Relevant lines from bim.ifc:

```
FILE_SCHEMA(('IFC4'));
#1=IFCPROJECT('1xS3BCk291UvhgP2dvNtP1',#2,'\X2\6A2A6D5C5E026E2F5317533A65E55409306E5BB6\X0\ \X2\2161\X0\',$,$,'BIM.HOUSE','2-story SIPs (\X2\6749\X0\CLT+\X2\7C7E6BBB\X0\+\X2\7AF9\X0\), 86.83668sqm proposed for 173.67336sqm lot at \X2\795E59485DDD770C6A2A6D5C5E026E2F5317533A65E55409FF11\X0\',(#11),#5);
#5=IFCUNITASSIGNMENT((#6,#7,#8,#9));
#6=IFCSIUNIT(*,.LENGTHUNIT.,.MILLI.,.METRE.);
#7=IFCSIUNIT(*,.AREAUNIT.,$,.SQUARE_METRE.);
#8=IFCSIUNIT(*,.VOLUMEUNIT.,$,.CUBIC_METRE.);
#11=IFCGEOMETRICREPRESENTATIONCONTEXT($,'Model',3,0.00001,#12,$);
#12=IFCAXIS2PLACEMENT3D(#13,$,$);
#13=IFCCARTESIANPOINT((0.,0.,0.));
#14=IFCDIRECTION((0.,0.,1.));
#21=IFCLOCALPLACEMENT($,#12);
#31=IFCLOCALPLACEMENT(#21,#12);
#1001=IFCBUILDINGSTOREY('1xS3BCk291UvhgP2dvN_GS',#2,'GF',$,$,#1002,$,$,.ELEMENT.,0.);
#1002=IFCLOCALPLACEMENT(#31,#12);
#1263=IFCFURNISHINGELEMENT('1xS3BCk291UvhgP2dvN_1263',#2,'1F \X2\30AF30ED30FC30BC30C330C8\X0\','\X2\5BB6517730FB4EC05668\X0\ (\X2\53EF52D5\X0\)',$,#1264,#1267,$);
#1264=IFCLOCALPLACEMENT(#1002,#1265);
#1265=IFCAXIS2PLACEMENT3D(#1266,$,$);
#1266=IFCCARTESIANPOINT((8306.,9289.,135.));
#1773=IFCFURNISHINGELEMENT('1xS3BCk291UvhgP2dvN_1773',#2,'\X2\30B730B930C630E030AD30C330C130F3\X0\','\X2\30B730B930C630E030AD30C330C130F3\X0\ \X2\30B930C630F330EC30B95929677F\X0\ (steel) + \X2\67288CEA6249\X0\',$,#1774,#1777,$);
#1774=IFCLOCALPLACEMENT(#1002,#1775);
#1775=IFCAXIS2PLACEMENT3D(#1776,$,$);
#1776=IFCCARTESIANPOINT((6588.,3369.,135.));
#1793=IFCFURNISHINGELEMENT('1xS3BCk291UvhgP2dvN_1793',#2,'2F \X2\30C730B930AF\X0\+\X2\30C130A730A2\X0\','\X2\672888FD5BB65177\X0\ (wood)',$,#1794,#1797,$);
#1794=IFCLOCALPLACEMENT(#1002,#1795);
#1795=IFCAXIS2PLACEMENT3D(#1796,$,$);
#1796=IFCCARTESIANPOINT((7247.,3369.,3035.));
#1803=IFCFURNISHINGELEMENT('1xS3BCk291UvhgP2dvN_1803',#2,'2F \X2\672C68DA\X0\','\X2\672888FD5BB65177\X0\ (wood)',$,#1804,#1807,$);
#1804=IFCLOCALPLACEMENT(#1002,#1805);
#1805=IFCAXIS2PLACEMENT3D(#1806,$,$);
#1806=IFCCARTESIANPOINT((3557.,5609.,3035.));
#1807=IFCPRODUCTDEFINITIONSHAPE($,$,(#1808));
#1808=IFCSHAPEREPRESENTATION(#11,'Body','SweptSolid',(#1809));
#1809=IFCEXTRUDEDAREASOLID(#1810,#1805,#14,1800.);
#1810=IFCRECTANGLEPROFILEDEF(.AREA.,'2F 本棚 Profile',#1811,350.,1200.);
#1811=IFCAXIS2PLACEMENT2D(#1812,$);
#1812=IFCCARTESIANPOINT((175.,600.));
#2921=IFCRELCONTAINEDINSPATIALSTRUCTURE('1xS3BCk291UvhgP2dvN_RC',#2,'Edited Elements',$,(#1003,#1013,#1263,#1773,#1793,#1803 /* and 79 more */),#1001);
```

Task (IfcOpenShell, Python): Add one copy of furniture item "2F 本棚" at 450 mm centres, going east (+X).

```python
import numpy as np
import ifcopenshell
import ifcopenshell.api.geometry
import ifcopenshell.api.root
import ifcopenshell.util.element
import ifcopenshell.util.placement
import ifcopenshell.util.unit

model = ifcopenshell.open("bim.ifc")
unit_scale = ifcopenshell.util.unit.calculate_unit_scale(model)


def reuse_history(source, copy):
    """copy_class also copies each property set's owner history, people and application; keep the originals."""
    for rel in copy.IsDefinedBy:
        if rel.is_a("IfcRelDefinesByProperties") and (history := rel.RelatingPropertyDefinition.OwnerHistory):
            rel.RelatingPropertyDefinition.OwnerHistory = source.OwnerHistory
            ifcopenshell.util.element.remove_deep2(model, history)


source = model.by_guid("1xS3BCk291UvhgP2dvN_1803")
base = ifcopenshell.util.placement.get_local_placement(source.ObjectPlacement)
step = np.array([1.0, 0.0, 0.0]) * 0.45 / unit_scale

for i in range(1, 2):
    copy = ifcopenshell.api.root.copy_class(model, product=source)
    copy.Representation = ifcopenshell.util.element.copy_deep(
        model, source.Representation, exclude=["IfcGeometricRepresentationContext", "IfcRepresentationMap"]
    )
    reuse_history(source, copy)
    matrix = base.copy()
    matrix[:3, 3] += i * step
    print("added at", matrix[:3, 3].round(3) + 0.0)
    ifcopenshell.api.geometry.edit_object_placement(model, product=copy, matrix=matrix, is_si=False)

model.write("bim_rev.ifc")
```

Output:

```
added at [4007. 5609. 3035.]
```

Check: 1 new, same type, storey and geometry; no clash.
